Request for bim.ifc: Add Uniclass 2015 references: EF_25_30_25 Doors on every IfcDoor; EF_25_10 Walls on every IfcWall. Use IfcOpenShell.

First a look at what the model holds.

```python
import ifcopenshell

model = ifcopenshell.open("bim.ifc")
print(model.schema)
print("classifications:", [c.Name for c in model.by_type("IfcClassification")])
for ifc_class in ("IfcDoor", "IfcRoof", "IfcStair", "IfcWall", "IfcWindow"):
    print(ifc_class, len(model.by_type(ifc_class)))
```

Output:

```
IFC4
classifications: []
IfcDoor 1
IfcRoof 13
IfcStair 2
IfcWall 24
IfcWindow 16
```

```python
import ifcopenshell
import ifcopenshell.api.classification

model = ifcopenshell.open("bim.ifc")

system = ifcopenshell.api.classification.add_classification(model, classification="Uniclass 2015")

codes = {
    "IfcDoor": ("EF_25_30_25", "Doors"),
    "IfcWall": ("EF_25_10", "Walls"),
}
for ifc_class, (code, name) in codes.items():
    products = model.by_type(ifc_class)
    ifcopenshell.api.classification.add_reference(
        model, products=products, classification=system, identification=code, name=name
    )
    print(code, len(products))

model.write("bim-out.ifc")
```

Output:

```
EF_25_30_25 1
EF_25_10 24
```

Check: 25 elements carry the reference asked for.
